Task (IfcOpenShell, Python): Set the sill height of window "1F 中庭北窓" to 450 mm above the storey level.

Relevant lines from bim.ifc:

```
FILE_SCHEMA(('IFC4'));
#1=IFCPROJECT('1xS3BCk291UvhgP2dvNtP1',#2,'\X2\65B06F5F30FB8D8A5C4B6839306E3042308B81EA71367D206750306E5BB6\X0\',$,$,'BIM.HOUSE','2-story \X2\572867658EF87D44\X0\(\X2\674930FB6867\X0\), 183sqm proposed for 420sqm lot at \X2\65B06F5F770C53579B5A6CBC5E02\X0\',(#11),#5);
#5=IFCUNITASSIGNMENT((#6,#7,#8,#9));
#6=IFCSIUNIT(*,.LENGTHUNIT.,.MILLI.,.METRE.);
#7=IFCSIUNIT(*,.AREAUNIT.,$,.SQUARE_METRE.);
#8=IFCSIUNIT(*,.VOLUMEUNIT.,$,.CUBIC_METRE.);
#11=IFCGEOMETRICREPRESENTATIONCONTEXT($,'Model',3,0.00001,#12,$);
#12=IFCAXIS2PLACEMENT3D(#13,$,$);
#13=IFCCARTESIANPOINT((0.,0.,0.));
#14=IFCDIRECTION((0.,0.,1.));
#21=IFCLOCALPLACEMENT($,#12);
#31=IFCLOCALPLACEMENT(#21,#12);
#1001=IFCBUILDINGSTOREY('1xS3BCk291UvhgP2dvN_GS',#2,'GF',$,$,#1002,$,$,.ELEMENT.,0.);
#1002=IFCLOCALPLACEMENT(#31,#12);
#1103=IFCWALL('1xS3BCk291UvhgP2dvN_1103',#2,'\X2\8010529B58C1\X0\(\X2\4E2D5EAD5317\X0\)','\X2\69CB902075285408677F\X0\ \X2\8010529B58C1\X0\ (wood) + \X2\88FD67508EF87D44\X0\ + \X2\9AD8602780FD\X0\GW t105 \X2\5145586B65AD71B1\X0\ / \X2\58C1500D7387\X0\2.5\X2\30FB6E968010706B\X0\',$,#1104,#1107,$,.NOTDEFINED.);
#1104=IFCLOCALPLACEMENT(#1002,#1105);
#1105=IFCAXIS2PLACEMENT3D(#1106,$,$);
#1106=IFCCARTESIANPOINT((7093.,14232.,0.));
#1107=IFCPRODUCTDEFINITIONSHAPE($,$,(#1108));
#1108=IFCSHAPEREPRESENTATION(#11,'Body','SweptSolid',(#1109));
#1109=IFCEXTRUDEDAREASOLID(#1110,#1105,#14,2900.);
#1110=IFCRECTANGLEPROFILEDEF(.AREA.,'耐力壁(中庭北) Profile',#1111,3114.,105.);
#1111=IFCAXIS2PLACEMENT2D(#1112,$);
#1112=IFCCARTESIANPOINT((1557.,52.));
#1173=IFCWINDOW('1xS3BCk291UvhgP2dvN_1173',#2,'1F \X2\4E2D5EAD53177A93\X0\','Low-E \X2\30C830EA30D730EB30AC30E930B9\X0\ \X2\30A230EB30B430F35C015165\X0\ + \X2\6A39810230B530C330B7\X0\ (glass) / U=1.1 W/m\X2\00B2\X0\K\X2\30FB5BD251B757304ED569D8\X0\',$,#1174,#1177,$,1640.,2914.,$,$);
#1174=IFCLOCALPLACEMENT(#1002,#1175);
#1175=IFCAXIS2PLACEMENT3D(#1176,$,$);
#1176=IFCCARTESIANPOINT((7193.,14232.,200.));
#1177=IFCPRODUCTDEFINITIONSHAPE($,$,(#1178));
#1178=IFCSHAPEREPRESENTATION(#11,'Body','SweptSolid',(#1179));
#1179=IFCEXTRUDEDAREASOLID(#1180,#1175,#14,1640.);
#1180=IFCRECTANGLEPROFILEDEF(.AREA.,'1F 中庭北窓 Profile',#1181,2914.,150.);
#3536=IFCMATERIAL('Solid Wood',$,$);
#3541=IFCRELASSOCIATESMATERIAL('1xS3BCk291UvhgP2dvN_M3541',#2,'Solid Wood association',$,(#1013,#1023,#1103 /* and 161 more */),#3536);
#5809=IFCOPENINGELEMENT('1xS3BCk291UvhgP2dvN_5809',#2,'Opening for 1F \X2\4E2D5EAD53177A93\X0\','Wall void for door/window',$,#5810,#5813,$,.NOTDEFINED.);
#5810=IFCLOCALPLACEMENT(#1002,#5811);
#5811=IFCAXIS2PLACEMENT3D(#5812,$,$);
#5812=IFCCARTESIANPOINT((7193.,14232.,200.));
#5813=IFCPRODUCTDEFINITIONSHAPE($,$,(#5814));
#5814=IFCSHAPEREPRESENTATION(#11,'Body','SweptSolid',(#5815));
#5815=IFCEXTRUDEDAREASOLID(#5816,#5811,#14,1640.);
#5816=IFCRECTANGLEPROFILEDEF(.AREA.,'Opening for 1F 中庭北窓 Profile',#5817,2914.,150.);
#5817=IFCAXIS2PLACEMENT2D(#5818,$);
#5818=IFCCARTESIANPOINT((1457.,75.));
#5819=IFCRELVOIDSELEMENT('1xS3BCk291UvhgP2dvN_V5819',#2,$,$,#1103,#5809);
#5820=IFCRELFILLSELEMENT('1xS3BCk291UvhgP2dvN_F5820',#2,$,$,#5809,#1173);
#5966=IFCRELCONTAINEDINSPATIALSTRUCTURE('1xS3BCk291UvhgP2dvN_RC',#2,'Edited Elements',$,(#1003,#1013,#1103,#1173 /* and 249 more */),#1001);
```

```python
import numpy as np
import ifcopenshell
import ifcopenshell.api.geometry
import ifcopenshell.geom
import ifcopenshell.util.element
import ifcopenshell.util.placement
import ifcopenshell.util.shape
import ifcopenshell.util.unit

model = ifcopenshell.open("bim.ifc")
unit_scale = ifcopenshell.util.unit.calculate_unit_scale(model)

window = model.by_guid("1xS3BCk291UvhgP2dvN_1173")
opening = window.FillsVoids[0].RelatingOpeningElement
storey = ifcopenshell.util.element.get_container(window, ifc_class="IfcBuildingStorey")
level = ifcopenshell.util.placement.get_local_placement(storey.ObjectPlacement)[2, 3]

# The opening's origin need not be at the sill, so measure its lowest point.
shape = ifcopenshell.geom.create_shape(ifcopenshell.geom.settings(), opening)
bottom = ifcopenshell.util.shape.get_shape_bottom_elevation(shape, shape.geometry) / unit_scale
dz = level + 0.45 / unit_scale - bottom

shift = np.array([0.0, 0.0, dz])
# The window is not placed relative to its opening, so move both.
for product in (opening, window):
    matrix = ifcopenshell.util.placement.get_local_placement(product.ObjectPlacement)
    matrix[:3, 3] += shift
    ifcopenshell.api.geometry.edit_object_placement(model, product=product, matrix=matrix, is_si=False)

print(f"moved by {dz * unit_scale:+.3f} m")

model.write("bim_updated.ifc")
```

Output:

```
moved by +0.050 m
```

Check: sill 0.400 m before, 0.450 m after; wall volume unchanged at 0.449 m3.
